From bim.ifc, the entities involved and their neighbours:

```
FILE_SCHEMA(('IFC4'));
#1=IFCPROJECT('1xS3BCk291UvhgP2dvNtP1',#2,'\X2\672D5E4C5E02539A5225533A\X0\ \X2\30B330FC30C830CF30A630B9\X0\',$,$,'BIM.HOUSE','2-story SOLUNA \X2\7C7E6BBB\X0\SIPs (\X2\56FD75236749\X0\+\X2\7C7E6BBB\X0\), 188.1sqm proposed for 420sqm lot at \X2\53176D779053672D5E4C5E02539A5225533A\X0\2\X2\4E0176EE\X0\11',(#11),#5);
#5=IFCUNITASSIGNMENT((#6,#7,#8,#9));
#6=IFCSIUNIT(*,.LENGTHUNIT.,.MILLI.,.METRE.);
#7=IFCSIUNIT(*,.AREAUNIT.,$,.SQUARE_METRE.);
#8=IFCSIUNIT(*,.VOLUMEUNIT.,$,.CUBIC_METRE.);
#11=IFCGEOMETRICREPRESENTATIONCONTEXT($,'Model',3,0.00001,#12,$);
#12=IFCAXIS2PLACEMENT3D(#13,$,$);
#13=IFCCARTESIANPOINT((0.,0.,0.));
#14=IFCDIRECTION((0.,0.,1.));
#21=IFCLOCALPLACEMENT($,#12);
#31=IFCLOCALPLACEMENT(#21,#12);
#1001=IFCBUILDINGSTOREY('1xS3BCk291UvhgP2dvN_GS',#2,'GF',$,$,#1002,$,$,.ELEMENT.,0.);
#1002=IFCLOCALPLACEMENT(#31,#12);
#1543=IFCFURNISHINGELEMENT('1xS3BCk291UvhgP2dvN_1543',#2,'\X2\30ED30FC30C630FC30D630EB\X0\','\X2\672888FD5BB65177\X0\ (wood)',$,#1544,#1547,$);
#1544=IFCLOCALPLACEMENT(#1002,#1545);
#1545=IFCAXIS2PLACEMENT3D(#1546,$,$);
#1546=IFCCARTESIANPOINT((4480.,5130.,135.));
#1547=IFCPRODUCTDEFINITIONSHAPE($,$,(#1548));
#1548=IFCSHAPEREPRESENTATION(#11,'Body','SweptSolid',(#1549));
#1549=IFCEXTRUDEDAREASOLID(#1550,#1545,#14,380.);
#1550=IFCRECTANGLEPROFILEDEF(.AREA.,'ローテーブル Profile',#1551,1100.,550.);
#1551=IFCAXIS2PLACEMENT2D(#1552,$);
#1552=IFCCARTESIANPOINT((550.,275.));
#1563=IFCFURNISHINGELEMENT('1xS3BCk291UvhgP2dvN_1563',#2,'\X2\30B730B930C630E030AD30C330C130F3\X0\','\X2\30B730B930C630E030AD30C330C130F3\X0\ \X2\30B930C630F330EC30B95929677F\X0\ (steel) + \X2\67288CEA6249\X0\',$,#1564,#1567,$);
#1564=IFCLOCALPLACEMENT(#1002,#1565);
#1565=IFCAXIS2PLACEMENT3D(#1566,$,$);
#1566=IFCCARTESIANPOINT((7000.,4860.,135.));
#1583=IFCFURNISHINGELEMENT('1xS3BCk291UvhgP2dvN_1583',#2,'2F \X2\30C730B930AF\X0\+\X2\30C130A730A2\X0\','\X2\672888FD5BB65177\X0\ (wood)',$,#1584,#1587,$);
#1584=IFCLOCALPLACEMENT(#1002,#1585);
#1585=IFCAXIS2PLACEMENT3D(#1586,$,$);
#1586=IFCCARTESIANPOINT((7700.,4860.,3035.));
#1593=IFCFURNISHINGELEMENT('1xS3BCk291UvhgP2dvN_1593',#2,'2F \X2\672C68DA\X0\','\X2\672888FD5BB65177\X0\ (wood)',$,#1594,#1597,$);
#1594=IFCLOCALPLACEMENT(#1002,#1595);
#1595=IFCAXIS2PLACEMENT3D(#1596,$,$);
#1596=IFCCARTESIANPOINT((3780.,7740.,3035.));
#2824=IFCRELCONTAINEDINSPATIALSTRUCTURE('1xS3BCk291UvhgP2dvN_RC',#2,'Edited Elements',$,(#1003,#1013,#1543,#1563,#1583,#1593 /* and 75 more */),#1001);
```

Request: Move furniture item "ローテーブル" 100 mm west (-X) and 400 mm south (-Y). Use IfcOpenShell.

```python
import ifcopenshell
import ifcopenshell.api.geometry
import ifcopenshell.util.placement
import ifcopenshell.util.unit

model = ifcopenshell.open("bim.ifc")
unit_scale = ifcopenshell.util.unit.calculate_unit_scale(model)

item = model.by_guid("1xS3BCk291UvhgP2dvN_1543")
matrix = ifcopenshell.util.placement.get_local_placement(item.ObjectPlacement)
matrix[0, 3] -= 0.1 / unit_scale
matrix[1, 3] -= 0.4 / unit_scale
ifcopenshell.api.geometry.edit_object_placement(model, product=item, matrix=matrix, is_si=False)

print(ifcopenshell.util.placement.get_local_placement(item.ObjectPlacement).round(3) + 0.0)

model.write("bim_rev.ifc")
```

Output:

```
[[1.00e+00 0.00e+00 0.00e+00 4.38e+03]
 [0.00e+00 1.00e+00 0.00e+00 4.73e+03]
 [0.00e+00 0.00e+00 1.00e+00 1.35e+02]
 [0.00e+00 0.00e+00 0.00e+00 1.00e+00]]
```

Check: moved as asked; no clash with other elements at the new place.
